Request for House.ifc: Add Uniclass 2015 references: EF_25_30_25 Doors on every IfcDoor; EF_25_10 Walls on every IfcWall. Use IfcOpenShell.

First a look at what the model holds.

```python
import ifcopenshell

model = ifcopenshell.open("House.ifc")
print(model.schema)
print("classifications:", [c.Name for c in model.by_type("IfcClassification")])
for ifc_class in ("IfcDoor", "IfcRoof", "IfcStair", "IfcWall", "IfcWindow"):
    print(ifc_class, len(model.by_type(ifc_class)))
```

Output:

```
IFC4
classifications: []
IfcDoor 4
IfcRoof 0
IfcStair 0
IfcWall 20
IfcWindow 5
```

```python
import ifcopenshell
import ifcopenshell.api.classification

model = ifcopenshell.open("House.ifc")

system = ifcopenshell.api.classification.add_classification(model, classification="Uniclass 2015")

codes = {
    "IfcDoor": ("EF_25_30_25", "Doors"),
    "IfcWall": ("EF_25_10", "Walls"),
}
for ifc_class, (code, name) in codes.items():
    products = model.by_type(ifc_class)
    ifcopenshell.api.classification.add_reference(
        model, products=products, classification=system, identification=code, name=name
    )
    print(code, len(products))

model.write("House-out.ifc")
```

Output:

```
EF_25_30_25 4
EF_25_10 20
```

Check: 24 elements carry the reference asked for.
